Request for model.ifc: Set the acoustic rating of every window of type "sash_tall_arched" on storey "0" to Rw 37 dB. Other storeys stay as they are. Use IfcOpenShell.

First a look at what the model holds.

```python
import ifcopenshell
import ifcopenshell.util.element

model = ifcopenshell.open("model.ifc")
print(model.schema)
storey = next(s for s in model.by_type("IfcBuildingStorey") if s.Name == "0")
windows = [e for e in ifcopenshell.util.element.get_decomposition(storey) if e.is_a("IfcWindow")]
seen = {}
for e in windows:
    element_type = ifcopenshell.util.element.get_type(e)
    key = (element_type.Name if element_type != e and element_type else None, ifcopenshell.util.element.get_pset(e, "Pset_WindowCommon", "AcousticRating"))
    seen[key] = seen.get(key, 0) + 1
for (name, value), count in sorted(seen.items(), key=str):
    print(count, "x", name, "|", value)
```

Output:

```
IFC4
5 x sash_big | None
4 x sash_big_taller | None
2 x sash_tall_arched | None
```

```python
import ifcopenshell
import ifcopenshell.api.pset
import ifcopenshell.util.element

model = ifcopenshell.open("model.ifc")

storey = next(s for s in model.by_type("IfcBuildingStorey") if s.Name == "0")
windows = [e for e in ifcopenshell.util.element.get_decomposition(storey) if e.is_a("IfcWindow")]

count = 0
for e in windows:
    element_type = ifcopenshell.util.element.get_type(e)
    if element_type in (None, e) or element_type.Name != "sash_tall_arched":
        continue
    # add_pset returns the element's existing set when there is one.
    pset = ifcopenshell.api.pset.add_pset(model, product=e, name="Pset_WindowCommon")
    ifcopenshell.api.pset.edit_pset(model, pset=pset, properties={"AcousticRating": "Rw 37 dB"})
    count += 1

print(count, "windows updated")

model.write("model_edited.ifc")
```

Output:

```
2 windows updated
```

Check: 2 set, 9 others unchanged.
